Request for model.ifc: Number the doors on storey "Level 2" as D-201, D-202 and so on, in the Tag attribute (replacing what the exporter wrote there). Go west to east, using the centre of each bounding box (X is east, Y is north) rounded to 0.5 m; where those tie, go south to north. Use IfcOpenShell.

First a look at what the model holds.

```python
import ifcopenshell
import ifcopenshell.util.element
import ifcopenshell.util.placement

model = ifcopenshell.open("model.ifc")
print(model.schema)
storey = next(s for s in model.by_type("IfcBuildingStorey") if s.Name == "Level 2")
doors = [e for e in ifcopenshell.util.element.get_decomposition(storey) if e.is_a("IfcDoor")]
for e in sorted(doors, key=lambda e: e.id()):
    origin = ifcopenshell.util.placement.get_local_placement(e.ObjectPlacement)[:3, 3]
    print(e.id(), e.Tag, e.Name, origin.round(2) + 0.0, sep=" | ")
```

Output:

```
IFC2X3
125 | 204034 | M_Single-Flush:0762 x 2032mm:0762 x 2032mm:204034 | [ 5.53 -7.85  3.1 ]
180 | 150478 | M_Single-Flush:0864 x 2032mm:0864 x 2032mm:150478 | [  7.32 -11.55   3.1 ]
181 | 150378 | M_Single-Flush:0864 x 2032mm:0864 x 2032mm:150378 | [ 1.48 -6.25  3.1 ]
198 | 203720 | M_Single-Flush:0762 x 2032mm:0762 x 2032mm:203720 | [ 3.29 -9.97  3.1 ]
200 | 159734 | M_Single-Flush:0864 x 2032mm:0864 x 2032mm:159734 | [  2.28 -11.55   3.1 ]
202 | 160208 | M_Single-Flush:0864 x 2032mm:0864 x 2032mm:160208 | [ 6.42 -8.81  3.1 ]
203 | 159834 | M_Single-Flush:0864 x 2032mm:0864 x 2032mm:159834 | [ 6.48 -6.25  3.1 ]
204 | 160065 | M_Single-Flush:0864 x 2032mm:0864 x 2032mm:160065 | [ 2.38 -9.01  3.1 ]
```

```python
import ifcopenshell
import ifcopenshell.geom
import ifcopenshell.util.element
import ifcopenshell.util.shape

model = ifcopenshell.open("model.ifc")
settings = ifcopenshell.geom.settings()
settings.set("use-world-coords", True)


def centre(element):
    shape = ifcopenshell.geom.create_shape(settings, element)
    return ifcopenshell.util.shape.get_bbox_centroid(shape.geometry)


storey = next(s for s in model.by_type("IfcBuildingStorey") if s.Name == "Level 2")
doors = [e for e in ifcopenshell.util.element.get_decomposition(storey) if e.is_a("IfcDoor")]

# Insertion points can sit at a corner or the storey origin, so sort by the geometry (in metres).
centres = {e: centre(e) for e in doors}
doors.sort(key=lambda e: (round(centres[e][0] / 0.5), centres[e][1]))

for i, e in enumerate(doors, start=1):
    number = f"D-2{i:02d}"
    e.Tag = number
    print(e.id(), number)

model.write("model_updated.ifc")
```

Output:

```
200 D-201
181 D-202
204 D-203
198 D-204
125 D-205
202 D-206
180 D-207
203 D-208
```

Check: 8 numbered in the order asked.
